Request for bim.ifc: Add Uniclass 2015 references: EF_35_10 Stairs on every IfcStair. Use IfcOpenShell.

First a look at what the model holds.

```python
import ifcopenshell

model = ifcopenshell.open("bim.ifc")
print(model.schema)
print("classifications:", [c.Name for c in model.by_type("IfcClassification")])
for ifc_class in ("IfcDoor", "IfcRoof", "IfcStair", "IfcWall", "IfcWindow"):
    print(ifc_class, len(model.by_type(ifc_class)))
```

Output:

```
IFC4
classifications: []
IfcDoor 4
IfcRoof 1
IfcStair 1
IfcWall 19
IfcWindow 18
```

```python
import ifcopenshell
import ifcopenshell.api.classification

model = ifcopenshell.open("bim.ifc")

system = ifcopenshell.api.classification.add_classification(model, classification="Uniclass 2015")

codes = {
    "IfcStair": ("EF_35_10", "Stairs"),
}
for ifc_class, (code, name) in codes.items():
    products = model.by_type(ifc_class)
    ifcopenshell.api.classification.add_reference(
        model, products=products, classification=system, identification=code, name=name
    )
    print(code, len(products))

model.write("bim_edited.ifc")
```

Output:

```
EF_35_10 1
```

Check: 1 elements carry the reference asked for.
